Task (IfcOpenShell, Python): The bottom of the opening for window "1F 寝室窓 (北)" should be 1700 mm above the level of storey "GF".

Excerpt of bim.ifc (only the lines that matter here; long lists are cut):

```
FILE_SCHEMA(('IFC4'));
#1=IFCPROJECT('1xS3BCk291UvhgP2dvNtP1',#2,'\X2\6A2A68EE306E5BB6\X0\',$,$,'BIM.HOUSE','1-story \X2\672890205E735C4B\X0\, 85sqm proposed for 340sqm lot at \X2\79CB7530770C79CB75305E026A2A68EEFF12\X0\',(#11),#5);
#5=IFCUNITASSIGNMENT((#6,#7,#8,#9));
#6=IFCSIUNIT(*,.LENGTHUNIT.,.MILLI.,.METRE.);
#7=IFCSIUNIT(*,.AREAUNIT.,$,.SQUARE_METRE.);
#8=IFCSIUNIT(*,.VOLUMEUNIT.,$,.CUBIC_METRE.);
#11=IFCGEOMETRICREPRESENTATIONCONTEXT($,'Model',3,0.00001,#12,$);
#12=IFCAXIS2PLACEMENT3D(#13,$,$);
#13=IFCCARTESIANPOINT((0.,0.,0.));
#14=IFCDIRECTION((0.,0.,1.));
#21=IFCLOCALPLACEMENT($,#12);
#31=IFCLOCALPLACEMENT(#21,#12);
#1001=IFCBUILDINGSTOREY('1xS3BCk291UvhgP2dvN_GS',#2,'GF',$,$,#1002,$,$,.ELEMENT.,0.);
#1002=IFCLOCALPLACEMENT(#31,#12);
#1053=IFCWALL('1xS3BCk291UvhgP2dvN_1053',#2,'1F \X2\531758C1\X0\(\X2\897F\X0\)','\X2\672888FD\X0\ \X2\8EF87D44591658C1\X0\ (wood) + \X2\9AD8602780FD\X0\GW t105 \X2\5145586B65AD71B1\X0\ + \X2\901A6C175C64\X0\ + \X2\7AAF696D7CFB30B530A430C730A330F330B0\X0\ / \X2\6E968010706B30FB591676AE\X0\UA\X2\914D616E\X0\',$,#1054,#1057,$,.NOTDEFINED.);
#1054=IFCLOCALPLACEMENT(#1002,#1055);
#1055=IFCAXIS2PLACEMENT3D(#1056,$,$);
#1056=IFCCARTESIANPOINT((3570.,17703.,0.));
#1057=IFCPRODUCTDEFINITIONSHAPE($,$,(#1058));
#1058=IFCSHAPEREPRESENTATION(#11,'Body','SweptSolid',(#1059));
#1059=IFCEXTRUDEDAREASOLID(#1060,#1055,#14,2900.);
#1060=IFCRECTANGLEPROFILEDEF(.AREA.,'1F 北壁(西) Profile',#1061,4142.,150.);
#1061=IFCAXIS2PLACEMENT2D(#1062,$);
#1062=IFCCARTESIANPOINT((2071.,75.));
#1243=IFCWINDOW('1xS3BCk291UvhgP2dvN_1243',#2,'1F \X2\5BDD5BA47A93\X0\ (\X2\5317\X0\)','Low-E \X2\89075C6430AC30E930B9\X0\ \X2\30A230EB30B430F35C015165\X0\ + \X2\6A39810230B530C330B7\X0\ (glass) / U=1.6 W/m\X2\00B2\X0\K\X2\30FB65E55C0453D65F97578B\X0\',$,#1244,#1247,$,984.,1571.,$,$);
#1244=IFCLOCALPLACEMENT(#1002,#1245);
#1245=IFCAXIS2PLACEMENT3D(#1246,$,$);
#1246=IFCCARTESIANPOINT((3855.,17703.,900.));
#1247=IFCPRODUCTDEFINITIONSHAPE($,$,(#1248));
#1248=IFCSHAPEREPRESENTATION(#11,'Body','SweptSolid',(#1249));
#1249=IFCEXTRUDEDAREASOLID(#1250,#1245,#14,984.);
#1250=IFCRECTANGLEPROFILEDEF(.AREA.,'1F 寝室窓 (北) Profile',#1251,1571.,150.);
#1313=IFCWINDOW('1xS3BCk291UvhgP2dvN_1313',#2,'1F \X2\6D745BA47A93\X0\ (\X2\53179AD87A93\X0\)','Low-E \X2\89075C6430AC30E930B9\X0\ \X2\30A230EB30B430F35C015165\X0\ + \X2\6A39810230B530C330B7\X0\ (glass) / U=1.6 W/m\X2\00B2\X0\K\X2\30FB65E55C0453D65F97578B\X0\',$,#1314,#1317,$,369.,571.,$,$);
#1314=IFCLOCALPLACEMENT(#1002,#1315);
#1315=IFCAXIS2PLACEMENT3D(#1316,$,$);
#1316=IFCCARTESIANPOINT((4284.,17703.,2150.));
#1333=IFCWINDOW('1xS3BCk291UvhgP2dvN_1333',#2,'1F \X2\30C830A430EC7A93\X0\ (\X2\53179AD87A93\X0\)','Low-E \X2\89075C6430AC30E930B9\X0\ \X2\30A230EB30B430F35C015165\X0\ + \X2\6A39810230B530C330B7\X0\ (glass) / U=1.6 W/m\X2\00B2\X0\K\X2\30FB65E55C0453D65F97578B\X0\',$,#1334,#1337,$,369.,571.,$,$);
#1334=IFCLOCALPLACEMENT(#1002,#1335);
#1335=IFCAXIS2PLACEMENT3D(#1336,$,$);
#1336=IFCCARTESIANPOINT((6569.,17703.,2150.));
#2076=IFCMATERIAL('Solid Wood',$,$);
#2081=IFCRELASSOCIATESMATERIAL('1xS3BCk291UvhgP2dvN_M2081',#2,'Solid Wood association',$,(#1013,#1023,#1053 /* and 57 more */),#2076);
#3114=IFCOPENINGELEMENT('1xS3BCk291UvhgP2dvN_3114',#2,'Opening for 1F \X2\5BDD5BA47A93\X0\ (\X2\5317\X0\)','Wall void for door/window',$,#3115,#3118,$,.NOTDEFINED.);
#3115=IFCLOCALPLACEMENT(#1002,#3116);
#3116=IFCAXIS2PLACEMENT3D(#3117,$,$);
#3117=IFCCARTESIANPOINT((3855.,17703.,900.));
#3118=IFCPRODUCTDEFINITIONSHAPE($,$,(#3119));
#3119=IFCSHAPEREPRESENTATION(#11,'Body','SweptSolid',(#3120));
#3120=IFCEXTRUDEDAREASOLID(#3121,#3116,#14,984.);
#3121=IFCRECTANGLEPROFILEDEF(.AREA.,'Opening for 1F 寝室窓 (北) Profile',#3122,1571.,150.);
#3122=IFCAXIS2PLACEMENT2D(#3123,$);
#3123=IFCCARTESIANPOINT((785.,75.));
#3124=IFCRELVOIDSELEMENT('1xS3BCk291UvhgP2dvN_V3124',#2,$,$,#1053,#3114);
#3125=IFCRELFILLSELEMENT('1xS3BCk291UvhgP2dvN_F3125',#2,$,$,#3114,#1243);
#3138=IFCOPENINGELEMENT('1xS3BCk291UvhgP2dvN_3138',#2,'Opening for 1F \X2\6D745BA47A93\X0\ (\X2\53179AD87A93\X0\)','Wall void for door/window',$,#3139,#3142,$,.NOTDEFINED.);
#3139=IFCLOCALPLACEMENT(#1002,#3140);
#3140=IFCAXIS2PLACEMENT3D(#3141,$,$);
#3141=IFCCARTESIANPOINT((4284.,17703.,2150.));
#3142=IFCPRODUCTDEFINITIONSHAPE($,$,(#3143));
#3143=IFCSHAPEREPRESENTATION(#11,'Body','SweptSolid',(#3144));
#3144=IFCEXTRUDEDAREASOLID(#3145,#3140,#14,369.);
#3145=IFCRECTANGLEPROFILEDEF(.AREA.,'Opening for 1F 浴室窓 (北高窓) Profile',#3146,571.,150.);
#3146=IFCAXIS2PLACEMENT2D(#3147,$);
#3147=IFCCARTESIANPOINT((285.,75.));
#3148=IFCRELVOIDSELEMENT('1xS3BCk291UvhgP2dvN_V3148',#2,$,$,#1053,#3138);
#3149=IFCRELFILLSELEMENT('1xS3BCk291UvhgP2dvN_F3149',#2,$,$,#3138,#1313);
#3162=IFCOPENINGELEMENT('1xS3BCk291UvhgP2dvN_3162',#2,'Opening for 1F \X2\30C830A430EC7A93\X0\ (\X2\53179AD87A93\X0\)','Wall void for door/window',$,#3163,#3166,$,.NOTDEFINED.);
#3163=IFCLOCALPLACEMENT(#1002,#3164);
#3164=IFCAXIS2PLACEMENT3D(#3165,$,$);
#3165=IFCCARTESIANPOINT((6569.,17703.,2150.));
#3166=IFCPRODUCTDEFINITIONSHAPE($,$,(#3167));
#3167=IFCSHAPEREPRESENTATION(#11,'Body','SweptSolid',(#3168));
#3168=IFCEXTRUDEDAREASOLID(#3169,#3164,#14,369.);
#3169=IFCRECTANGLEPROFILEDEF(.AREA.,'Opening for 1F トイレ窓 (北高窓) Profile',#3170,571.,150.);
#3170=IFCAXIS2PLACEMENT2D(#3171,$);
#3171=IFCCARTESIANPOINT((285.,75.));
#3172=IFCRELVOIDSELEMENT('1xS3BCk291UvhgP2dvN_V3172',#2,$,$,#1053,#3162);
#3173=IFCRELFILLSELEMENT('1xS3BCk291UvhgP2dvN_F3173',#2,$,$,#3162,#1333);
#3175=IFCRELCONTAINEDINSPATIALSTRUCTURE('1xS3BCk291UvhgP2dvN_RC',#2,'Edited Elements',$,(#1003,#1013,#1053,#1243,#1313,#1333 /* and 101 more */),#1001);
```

```python
import numpy as np
import ifcopenshell
import ifcopenshell.api.geometry
import ifcopenshell.geom
import ifcopenshell.util.element
import ifcopenshell.util.placement
import ifcopenshell.util.shape
import ifcopenshell.util.unit

model = ifcopenshell.open("bim.ifc")
unit_scale = ifcopenshell.util.unit.calculate_unit_scale(model)

window = model.by_id(1243)
opening = window.FillsVoids[0].RelatingOpeningElement
storey = ifcopenshell.util.element.get_container(window, ifc_class="IfcBuildingStorey")
level = ifcopenshell.util.placement.get_local_placement(storey.ObjectPlacement)[2, 3]

# The opening's origin need not be at the sill, so measure its lowest point.
shape = ifcopenshell.geom.create_shape(ifcopenshell.geom.settings(), opening)
bottom = ifcopenshell.util.shape.get_shape_bottom_elevation(shape, shape.geometry) / unit_scale
dz = level + 1.7 / unit_scale - bottom

shift = np.array([0.0, 0.0, dz])
# The window is not placed relative to its opening, so move both.
for product in (opening, window):
    matrix = ifcopenshell.util.placement.get_local_placement(product.ObjectPlacement)
    matrix[:3, 3] += shift
    ifcopenshell.api.geometry.edit_object_placement(model, product=product, matrix=matrix, is_si=False)

print(f"moved by {dz * unit_scale:+.3f} m")

model.write("bim-out.ifc")
```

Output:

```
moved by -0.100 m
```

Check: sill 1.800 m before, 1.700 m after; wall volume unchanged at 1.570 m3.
